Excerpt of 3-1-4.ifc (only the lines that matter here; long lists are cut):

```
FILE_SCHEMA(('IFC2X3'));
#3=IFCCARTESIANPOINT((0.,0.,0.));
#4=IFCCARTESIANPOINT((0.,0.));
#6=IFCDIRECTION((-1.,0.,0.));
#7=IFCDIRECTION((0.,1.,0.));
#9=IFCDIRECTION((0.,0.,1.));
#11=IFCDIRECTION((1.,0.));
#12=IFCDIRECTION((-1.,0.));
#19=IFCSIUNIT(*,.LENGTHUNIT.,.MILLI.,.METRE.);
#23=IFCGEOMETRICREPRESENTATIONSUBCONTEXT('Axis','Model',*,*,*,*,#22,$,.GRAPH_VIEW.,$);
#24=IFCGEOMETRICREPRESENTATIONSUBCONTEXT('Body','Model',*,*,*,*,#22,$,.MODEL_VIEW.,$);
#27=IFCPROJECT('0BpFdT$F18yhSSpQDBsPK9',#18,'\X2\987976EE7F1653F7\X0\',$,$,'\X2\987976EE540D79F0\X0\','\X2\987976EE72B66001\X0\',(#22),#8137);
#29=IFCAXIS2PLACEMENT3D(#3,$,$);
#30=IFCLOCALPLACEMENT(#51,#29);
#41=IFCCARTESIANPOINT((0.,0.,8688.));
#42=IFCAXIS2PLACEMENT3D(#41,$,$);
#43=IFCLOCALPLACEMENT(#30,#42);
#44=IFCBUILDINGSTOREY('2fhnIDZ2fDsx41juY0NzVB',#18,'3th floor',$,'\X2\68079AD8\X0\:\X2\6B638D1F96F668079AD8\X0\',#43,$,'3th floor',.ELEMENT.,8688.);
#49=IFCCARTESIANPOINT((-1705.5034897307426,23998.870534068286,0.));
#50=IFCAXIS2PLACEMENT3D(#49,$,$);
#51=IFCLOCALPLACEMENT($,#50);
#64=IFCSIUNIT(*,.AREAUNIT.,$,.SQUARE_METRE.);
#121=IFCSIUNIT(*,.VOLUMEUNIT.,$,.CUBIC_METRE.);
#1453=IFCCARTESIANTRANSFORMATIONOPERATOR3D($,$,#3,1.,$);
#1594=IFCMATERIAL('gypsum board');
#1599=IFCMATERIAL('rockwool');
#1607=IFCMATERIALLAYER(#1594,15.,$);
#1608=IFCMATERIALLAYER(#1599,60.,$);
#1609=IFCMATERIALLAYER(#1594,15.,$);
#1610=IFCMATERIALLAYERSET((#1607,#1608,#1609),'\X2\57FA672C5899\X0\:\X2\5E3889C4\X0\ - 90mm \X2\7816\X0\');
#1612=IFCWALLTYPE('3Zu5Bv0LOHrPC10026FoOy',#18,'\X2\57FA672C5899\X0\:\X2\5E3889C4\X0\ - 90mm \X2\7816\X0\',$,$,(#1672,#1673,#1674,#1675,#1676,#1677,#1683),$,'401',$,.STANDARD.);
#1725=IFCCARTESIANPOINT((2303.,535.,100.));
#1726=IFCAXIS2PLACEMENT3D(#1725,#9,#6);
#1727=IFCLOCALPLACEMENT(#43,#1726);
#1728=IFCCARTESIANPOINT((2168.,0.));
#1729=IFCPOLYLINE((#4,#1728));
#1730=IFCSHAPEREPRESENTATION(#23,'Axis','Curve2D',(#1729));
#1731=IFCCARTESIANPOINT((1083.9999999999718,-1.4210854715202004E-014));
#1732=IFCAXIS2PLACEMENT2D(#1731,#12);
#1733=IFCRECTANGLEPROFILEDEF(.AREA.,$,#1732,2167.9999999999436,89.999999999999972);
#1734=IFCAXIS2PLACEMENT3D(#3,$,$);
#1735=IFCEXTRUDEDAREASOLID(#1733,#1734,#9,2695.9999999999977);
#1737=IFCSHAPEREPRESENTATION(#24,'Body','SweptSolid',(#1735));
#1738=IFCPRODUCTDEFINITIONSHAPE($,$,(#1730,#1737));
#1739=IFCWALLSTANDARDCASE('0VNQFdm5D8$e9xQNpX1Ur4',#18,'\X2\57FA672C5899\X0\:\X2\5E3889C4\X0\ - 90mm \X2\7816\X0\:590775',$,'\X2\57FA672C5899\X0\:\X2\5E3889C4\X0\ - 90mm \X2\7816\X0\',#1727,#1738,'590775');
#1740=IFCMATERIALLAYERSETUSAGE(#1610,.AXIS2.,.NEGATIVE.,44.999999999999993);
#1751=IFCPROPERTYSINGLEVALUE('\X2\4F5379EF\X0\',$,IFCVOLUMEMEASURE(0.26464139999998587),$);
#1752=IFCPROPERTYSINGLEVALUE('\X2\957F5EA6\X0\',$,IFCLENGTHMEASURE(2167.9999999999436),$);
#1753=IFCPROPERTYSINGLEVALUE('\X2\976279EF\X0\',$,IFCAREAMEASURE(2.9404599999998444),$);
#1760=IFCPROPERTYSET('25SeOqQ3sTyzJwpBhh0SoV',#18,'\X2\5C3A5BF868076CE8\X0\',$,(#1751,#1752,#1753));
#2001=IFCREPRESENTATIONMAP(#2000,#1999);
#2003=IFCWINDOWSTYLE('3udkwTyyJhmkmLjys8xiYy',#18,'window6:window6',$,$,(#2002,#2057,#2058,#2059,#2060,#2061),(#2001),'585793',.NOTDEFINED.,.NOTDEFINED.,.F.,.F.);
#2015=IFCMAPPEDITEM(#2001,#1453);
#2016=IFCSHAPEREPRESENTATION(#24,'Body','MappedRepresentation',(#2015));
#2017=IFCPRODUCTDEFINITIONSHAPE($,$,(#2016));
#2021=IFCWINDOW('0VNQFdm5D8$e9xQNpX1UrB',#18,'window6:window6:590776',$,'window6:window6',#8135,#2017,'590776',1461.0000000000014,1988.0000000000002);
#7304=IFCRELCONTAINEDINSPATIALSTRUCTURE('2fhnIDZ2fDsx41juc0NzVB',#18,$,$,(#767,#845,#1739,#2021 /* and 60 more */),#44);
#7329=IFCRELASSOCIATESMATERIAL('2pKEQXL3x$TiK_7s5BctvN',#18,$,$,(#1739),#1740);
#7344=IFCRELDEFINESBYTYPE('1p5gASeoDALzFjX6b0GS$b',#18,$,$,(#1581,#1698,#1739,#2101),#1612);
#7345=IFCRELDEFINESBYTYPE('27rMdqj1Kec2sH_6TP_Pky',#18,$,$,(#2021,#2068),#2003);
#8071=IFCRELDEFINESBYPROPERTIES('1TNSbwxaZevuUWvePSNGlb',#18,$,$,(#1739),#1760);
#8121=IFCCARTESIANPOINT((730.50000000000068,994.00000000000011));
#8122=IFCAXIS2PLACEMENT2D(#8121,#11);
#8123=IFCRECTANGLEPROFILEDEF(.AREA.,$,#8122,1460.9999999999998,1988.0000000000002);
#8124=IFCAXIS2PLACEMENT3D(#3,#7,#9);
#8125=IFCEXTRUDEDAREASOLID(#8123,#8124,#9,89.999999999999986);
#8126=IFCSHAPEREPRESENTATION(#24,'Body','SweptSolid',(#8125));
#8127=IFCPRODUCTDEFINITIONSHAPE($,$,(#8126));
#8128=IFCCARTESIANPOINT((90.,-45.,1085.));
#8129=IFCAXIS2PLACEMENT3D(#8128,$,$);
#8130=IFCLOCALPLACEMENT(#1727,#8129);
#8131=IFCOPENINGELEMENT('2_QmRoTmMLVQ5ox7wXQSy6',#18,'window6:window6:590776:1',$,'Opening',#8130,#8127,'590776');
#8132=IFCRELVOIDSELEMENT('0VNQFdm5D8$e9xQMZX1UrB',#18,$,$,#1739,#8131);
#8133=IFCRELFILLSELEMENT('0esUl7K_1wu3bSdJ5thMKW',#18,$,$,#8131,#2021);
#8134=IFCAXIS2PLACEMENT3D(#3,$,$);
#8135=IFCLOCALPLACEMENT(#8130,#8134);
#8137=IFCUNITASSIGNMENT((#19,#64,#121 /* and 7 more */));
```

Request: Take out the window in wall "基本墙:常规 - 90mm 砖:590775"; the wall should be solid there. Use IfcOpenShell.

```python
import ifcopenshell
import ifcopenshell.api.feature
import ifcopenshell.api.pset
import ifcopenshell.api.root
import ifcopenshell.geom
import ifcopenshell.util.element
import ifcopenshell.util.shape
import ifcopenshell.util.unit

model = ifcopenshell.open("3-1-4.ifc")
area_scale = ifcopenshell.util.unit.calculate_unit_scale(model, "AREAUNIT")
volume_scale = ifcopenshell.util.unit.calculate_unit_scale(model, "VOLUMEUNIT")
settings = ifcopenshell.geom.settings()


def volume(element):
    """Net volume in cubic metres, openings subtracted."""
    shape = ifcopenshell.geom.create_shape(settings, element)
    return ifcopenshell.util.shape.get_volume(shape.geometry)


window = model.by_guid("0VNQFdm5D8$e9xQNpX1UrB")
opening = window.FillsVoids[0].RelatingOpeningElement
wall = opening.VoidsElements[0].RelatingBuildingElement
before = volume(wall)

ifcopenshell.api.root.remove_product(model, product=window)
ifcopenshell.api.feature.remove_feature(model, feature=opening)

after = volume(wall)
thickness = 0.09  # wall thickness in metres

# Update the wall's stored quantities.
pset = model.by_id(ifcopenshell.util.element.get_pset(wall, "尺寸标注", should_inherit=False)["id"])
ifcopenshell.api.pset.edit_pset(model, pset=pset, properties={
    "体积": model.create_entity("IfcVolumeMeasure", after / volume_scale),
    "面积": model.create_entity("IfcAreaMeasure", after / thickness / area_scale),
})

print(f"wall volume {before:.3f} -> {after:.3f} m3")

model.write("3-1-4_v2.ifc")
```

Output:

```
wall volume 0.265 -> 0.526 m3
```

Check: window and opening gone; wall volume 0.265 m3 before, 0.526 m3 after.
